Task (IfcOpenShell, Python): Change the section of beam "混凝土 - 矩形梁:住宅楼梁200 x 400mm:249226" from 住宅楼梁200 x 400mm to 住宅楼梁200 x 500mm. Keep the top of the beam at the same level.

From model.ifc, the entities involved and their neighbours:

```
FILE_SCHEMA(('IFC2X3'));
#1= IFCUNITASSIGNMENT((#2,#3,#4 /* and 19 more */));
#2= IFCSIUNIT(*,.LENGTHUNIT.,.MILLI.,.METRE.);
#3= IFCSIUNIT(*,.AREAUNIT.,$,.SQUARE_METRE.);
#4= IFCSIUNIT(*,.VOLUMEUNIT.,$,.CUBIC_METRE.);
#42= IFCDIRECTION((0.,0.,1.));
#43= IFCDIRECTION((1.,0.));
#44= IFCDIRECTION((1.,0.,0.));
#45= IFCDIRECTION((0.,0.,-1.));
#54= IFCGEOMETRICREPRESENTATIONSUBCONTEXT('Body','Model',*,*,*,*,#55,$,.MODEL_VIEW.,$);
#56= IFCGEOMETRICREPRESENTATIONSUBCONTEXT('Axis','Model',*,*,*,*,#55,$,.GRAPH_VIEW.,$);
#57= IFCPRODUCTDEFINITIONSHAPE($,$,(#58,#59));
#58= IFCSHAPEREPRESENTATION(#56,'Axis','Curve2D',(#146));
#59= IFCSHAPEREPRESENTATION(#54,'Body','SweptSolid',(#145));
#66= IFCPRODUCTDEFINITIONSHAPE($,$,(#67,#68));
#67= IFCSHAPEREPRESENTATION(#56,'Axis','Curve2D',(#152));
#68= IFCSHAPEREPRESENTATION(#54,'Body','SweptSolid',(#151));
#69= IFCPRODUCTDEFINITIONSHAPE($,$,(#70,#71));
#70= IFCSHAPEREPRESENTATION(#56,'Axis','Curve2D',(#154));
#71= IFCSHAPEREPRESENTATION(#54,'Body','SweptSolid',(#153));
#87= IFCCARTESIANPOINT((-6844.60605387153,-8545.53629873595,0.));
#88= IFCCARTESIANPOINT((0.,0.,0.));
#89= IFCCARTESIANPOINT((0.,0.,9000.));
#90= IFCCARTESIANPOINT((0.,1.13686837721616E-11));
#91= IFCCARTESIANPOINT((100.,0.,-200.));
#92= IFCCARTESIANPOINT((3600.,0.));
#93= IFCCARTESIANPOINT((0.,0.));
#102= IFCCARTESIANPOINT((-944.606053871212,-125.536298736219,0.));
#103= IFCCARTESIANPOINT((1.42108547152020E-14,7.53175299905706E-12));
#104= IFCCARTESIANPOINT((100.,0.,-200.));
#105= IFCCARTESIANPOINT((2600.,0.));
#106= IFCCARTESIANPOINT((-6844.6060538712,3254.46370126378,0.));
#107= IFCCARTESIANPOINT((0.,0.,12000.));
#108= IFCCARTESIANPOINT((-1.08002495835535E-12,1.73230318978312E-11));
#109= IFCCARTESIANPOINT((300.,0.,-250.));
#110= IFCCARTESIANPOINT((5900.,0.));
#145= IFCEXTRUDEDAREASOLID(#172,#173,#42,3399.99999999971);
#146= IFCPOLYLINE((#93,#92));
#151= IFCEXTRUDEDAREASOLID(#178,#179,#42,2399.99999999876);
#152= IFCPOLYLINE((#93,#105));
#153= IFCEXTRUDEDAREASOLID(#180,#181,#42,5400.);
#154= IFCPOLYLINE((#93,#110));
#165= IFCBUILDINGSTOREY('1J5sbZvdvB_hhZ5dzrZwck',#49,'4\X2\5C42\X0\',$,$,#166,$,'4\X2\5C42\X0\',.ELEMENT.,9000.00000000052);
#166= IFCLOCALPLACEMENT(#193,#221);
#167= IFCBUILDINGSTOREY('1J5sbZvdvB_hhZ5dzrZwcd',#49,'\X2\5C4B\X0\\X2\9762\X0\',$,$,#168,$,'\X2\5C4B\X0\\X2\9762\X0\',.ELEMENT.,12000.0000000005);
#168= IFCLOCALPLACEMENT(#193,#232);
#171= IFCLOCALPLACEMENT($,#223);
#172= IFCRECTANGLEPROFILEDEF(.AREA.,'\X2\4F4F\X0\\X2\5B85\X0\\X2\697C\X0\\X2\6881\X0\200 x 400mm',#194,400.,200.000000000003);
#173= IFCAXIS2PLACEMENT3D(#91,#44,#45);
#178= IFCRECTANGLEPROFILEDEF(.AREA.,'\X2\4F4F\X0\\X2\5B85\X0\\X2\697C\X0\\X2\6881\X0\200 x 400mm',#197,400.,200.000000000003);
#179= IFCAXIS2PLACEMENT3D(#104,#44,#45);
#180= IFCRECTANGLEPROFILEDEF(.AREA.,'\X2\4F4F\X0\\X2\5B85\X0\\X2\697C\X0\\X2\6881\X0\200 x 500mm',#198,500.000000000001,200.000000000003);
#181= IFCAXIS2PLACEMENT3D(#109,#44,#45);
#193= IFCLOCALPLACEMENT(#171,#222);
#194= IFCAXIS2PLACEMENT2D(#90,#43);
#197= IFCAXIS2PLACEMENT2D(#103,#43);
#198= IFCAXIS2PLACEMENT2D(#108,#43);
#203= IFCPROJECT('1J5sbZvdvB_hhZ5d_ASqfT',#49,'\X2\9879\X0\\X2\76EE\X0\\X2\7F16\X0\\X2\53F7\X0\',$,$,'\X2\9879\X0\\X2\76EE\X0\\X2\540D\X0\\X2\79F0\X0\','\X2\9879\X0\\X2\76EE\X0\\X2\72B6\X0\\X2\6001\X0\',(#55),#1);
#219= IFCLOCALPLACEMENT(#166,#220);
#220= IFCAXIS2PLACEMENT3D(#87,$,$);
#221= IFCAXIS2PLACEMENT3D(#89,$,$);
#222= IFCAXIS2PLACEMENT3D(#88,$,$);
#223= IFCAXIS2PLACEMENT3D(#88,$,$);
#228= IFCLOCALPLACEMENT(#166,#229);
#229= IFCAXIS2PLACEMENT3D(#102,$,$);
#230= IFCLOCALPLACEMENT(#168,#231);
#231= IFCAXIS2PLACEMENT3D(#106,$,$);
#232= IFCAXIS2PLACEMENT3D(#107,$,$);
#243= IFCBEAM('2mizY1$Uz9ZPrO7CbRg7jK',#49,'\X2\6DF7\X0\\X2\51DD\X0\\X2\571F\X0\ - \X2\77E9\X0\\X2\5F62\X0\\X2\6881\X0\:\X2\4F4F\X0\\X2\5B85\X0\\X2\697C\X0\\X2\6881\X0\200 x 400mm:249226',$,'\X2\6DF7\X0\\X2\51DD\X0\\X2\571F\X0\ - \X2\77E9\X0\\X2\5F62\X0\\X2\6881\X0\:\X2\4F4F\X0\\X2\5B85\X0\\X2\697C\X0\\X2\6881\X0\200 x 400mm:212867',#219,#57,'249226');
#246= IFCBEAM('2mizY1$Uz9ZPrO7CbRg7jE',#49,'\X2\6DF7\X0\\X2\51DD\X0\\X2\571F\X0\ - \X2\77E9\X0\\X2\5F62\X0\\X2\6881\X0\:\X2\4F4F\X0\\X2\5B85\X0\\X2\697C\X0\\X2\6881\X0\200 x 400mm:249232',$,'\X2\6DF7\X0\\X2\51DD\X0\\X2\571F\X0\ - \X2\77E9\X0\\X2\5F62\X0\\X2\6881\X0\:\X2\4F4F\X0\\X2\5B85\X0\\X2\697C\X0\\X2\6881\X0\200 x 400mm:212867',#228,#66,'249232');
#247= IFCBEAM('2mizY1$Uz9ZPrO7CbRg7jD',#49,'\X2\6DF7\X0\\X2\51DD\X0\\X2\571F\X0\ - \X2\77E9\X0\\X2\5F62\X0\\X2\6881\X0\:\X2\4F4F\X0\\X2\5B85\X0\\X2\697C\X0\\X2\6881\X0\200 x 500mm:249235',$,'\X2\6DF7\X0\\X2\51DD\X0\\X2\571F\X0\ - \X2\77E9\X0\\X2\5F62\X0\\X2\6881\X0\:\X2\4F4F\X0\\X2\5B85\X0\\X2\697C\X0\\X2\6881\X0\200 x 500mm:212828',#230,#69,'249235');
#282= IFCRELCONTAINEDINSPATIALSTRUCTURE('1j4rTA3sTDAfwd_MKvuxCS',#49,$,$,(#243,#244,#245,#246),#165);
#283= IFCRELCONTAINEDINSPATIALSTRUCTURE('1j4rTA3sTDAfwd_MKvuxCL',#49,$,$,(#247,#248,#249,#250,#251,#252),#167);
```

```python
import ifcopenshell
import ifcopenshell.util.element
import ifcopenshell.util.representation

model = ifcopenshell.open("model.ifc")

member = model.by_guid("2mizY1$Uz9ZPrO7CbRg7jK")
source = next(p for p in model.by_type("IfcRectangleProfileDef") if p.ProfileName == "住宅楼梁200 x 500mm")

body = ifcopenshell.util.representation.get_representation(member, "Model", "Body")
solid = body.Items[0]
old_profile = solid.SweptArea

# Copy the section's sizes but keep this member's own profile position.
profile = ifcopenshell.util.element.copy(model, source)
# Profiles are centred, so shift by half the change in depth to hold the top.
shift = (old_profile.XDim - profile.XDim) / 2
x, y = old_profile.Position.Location.Coordinates
up = (-1.0, 0.0)  # upwards, in the solid's own plane
location = model.createIfcCartesianPoint((x + up[0] * shift, y + up[1] * shift))
profile.Position = model.createIfcAxis2Placement2D(location, old_profile.Position.RefDirection)
solid.SweptArea = profile
if not model.get_total_inverses(old_profile):
    ifcopenshell.util.element.remove_deep2(model, old_profile)
member.Name = member.Name.replace("住宅楼梁200 x 400mm", "住宅楼梁200 x 500mm")
member.ObjectType = member.ObjectType.replace("住宅楼梁200 x 400mm", "住宅楼梁200 x 500mm")

print(solid.SweptArea)

model.write("model-out.ifc")
```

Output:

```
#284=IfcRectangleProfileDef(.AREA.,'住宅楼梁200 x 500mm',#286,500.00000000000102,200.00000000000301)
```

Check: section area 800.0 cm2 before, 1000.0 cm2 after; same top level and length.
